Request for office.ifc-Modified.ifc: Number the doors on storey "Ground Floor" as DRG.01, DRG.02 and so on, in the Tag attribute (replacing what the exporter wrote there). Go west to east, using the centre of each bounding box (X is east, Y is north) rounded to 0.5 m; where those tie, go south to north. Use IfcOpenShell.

First a look at what the model holds.

```python
import ifcopenshell
import ifcopenshell.util.element
import ifcopenshell.util.placement

model = ifcopenshell.open("office.ifc-Modified.ifc")
print(model.schema)
storey = next(s for s in model.by_type("IfcBuildingStorey") if s.Name == "Ground Floor")
doors = [e for e in ifcopenshell.util.element.get_decomposition(storey) if e.is_a("IfcDoor")]
for e in sorted(doors, key=lambda e: e.id()):
    origin = ifcopenshell.util.placement.get_local_placement(e.ObjectPlacement)[:3, 3]
    print(e.id(), e.Tag, e.Name, origin.round(2) + 0.0, sep=" | ")
```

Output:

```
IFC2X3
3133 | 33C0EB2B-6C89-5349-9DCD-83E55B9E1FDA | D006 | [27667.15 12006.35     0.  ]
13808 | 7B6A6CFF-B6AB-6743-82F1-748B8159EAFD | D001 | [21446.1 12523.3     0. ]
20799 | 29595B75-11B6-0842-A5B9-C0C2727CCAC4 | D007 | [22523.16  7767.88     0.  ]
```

```python
import ifcopenshell
import ifcopenshell.geom
import ifcopenshell.util.element
import ifcopenshell.util.shape

model = ifcopenshell.open("office.ifc-Modified.ifc")
settings = ifcopenshell.geom.settings()
settings.set("use-world-coords", True)


def centre(element):
    shape = ifcopenshell.geom.create_shape(settings, element)
    return ifcopenshell.util.shape.get_bbox_centroid(shape.geometry)


storey = next(s for s in model.by_type("IfcBuildingStorey") if s.Name == "Ground Floor")
doors = [e for e in ifcopenshell.util.element.get_decomposition(storey) if e.is_a("IfcDoor")]

# Insertion points can sit at a corner or the storey origin, so sort by the geometry (in metres).
centres = {e: centre(e) for e in doors}
doors.sort(key=lambda e: (round(centres[e][0] / 0.5), centres[e][1]))

for i, e in enumerate(doors, start=1):
    number = f"DRG.{i:02d}"
    e.Tag = number
    print(e.id(), number)

model.write("office.ifc-Modified-out.ifc")
```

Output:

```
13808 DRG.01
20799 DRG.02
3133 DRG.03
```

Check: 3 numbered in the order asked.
